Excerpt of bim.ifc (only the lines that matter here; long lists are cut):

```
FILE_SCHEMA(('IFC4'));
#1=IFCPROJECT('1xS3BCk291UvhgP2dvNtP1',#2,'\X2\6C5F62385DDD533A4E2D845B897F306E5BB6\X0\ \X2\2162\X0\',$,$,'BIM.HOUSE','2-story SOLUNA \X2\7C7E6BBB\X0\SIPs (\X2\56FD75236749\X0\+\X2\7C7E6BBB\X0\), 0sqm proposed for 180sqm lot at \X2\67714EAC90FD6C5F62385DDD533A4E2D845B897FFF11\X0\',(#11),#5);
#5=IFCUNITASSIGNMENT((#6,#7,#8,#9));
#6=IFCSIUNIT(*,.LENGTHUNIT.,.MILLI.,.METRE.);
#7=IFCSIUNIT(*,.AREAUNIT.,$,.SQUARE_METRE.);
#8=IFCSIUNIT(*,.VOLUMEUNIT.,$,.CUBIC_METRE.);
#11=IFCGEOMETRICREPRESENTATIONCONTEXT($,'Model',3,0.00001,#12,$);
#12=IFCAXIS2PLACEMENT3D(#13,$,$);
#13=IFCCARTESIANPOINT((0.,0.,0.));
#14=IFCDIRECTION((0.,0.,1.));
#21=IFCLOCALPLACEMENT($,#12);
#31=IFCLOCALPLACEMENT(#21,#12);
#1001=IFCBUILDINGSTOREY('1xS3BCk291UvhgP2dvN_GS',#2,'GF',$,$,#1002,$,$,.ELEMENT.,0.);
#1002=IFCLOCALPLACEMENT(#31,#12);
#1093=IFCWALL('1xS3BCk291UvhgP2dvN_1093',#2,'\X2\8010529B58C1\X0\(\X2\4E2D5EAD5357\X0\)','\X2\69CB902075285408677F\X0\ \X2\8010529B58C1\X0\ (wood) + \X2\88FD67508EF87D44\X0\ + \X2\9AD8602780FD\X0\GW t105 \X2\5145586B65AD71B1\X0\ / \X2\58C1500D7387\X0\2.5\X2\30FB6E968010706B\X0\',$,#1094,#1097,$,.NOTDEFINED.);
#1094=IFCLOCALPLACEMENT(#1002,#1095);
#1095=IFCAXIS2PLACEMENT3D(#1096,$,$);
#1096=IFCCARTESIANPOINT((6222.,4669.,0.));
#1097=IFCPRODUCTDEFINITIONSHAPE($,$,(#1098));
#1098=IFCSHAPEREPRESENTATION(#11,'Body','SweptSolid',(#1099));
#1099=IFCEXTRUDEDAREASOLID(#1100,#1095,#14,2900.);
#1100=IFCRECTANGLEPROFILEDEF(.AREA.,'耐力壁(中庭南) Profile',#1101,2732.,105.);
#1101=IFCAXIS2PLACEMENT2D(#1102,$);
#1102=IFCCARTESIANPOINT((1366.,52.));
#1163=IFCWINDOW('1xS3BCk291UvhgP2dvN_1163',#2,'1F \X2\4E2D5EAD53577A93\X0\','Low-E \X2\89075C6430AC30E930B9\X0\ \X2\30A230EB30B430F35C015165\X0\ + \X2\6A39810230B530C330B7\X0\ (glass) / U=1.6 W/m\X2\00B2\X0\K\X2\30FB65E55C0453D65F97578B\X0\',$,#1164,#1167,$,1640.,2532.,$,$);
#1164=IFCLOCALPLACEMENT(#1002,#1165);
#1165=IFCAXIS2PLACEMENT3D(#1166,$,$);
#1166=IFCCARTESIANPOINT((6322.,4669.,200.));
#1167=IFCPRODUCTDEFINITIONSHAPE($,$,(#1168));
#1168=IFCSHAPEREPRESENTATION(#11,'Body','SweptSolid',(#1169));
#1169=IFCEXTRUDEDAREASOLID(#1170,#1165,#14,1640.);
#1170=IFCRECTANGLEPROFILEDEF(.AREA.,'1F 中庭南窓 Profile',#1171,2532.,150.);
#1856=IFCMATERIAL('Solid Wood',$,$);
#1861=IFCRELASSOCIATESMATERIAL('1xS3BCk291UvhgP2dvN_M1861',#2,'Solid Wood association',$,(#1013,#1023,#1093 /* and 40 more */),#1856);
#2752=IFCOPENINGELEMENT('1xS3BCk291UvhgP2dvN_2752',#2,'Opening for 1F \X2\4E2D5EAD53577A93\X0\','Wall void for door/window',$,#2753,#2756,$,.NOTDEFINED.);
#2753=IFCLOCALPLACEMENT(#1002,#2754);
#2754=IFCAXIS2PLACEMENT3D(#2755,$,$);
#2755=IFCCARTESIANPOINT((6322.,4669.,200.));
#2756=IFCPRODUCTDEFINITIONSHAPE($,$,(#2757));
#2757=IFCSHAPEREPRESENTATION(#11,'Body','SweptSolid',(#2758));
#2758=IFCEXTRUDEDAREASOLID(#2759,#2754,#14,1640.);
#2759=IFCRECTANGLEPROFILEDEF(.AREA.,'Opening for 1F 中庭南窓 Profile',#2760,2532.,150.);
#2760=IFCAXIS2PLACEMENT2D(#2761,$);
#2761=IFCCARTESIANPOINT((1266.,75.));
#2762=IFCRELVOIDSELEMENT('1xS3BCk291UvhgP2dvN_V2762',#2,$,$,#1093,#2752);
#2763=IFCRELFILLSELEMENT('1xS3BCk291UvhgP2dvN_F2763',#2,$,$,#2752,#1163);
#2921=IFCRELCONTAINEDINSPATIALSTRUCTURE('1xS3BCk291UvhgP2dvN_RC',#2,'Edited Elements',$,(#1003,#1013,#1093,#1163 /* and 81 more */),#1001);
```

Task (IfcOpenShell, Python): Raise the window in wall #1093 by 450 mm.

```python
import numpy as np
import ifcopenshell
import ifcopenshell.api.geometry
import ifcopenshell.util.placement
import ifcopenshell.util.unit

model = ifcopenshell.open("bim.ifc")
unit_scale = ifcopenshell.util.unit.calculate_unit_scale(model)

window = model.by_id(1163)
opening = window.FillsVoids[0].RelatingOpeningElement
dz = 0.45 / unit_scale

shift = np.array([0.0, 0.0, dz])
# The window is not placed relative to its opening, so move both.
for product in (opening, window):
    matrix = ifcopenshell.util.placement.get_local_placement(product.ObjectPlacement)
    matrix[:3, 3] += shift
    ifcopenshell.api.geometry.edit_object_placement(model, product=product, matrix=matrix, is_si=False)

print(f"moved by {dz * unit_scale:+.3f} m")

model.write("bim_updated.ifc")
```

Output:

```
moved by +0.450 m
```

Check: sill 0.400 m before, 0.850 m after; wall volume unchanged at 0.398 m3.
